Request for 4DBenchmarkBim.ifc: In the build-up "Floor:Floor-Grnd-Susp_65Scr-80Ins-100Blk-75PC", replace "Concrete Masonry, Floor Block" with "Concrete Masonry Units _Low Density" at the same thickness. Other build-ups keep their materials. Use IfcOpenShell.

First a look at what the model holds.

```python
import ifcopenshell
import ifcopenshell.util.element

model = ifcopenshell.open("4DBenchmarkBim.ifc")
print(model.schema)
for layer_set in model.by_type("IfcMaterialLayerSet"):
    if layer_set.LayerSetName == "Floor:Floor-Grnd-Susp_65Scr-80Ins-100Blk-75PC":
        for layer in layer_set.MaterialLayers:
            print(layer.id(), layer.Material and layer.Material.Name, layer.LayerThickness, sep=" | ")
        print(len(ifcopenshell.util.element.get_elements_by_material(model, layer_set)), "elements and types use it")
print(sorted(m.Name for m in model.by_type("IfcMaterial") if m.Name)[:60])
```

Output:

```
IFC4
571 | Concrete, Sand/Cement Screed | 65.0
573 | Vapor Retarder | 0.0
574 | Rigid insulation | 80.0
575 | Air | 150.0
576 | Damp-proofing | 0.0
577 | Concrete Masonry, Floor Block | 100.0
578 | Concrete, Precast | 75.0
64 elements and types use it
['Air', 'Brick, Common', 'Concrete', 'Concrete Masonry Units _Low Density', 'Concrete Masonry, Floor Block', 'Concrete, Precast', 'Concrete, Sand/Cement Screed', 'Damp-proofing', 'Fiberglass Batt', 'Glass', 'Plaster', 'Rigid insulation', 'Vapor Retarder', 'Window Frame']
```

```python
import ifcopenshell
import ifcopenshell.api.material

model = ifcopenshell.open("4DBenchmarkBim.ifc")

layer_set = next(s for s in model.by_type("IfcMaterialLayerSet") if s.LayerSetName == "Floor:Floor-Grnd-Susp_65Scr-80Ins-100Blk-75PC")
layer = next(l for l in layer_set.MaterialLayers if l.Material and l.Material.Name == "Concrete Masonry, Floor Block")
material = next(m for m in model.by_type("IfcMaterial") if m.Name == "Concrete Masonry Units _Low Density")

# Point this one layer at the other material; renaming the old one would change it everywhere.
ifcopenshell.api.material.edit_layer(model, layer=layer, attributes={"Name": material.Name}, material=material)

print([l.Material.Name if l.Material else None for l in layer_set.MaterialLayers])

model.write("4DBenchmarkBim-out.ifc")
```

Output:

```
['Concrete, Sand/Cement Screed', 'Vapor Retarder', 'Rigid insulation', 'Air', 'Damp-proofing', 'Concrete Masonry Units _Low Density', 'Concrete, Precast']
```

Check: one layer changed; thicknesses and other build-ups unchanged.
